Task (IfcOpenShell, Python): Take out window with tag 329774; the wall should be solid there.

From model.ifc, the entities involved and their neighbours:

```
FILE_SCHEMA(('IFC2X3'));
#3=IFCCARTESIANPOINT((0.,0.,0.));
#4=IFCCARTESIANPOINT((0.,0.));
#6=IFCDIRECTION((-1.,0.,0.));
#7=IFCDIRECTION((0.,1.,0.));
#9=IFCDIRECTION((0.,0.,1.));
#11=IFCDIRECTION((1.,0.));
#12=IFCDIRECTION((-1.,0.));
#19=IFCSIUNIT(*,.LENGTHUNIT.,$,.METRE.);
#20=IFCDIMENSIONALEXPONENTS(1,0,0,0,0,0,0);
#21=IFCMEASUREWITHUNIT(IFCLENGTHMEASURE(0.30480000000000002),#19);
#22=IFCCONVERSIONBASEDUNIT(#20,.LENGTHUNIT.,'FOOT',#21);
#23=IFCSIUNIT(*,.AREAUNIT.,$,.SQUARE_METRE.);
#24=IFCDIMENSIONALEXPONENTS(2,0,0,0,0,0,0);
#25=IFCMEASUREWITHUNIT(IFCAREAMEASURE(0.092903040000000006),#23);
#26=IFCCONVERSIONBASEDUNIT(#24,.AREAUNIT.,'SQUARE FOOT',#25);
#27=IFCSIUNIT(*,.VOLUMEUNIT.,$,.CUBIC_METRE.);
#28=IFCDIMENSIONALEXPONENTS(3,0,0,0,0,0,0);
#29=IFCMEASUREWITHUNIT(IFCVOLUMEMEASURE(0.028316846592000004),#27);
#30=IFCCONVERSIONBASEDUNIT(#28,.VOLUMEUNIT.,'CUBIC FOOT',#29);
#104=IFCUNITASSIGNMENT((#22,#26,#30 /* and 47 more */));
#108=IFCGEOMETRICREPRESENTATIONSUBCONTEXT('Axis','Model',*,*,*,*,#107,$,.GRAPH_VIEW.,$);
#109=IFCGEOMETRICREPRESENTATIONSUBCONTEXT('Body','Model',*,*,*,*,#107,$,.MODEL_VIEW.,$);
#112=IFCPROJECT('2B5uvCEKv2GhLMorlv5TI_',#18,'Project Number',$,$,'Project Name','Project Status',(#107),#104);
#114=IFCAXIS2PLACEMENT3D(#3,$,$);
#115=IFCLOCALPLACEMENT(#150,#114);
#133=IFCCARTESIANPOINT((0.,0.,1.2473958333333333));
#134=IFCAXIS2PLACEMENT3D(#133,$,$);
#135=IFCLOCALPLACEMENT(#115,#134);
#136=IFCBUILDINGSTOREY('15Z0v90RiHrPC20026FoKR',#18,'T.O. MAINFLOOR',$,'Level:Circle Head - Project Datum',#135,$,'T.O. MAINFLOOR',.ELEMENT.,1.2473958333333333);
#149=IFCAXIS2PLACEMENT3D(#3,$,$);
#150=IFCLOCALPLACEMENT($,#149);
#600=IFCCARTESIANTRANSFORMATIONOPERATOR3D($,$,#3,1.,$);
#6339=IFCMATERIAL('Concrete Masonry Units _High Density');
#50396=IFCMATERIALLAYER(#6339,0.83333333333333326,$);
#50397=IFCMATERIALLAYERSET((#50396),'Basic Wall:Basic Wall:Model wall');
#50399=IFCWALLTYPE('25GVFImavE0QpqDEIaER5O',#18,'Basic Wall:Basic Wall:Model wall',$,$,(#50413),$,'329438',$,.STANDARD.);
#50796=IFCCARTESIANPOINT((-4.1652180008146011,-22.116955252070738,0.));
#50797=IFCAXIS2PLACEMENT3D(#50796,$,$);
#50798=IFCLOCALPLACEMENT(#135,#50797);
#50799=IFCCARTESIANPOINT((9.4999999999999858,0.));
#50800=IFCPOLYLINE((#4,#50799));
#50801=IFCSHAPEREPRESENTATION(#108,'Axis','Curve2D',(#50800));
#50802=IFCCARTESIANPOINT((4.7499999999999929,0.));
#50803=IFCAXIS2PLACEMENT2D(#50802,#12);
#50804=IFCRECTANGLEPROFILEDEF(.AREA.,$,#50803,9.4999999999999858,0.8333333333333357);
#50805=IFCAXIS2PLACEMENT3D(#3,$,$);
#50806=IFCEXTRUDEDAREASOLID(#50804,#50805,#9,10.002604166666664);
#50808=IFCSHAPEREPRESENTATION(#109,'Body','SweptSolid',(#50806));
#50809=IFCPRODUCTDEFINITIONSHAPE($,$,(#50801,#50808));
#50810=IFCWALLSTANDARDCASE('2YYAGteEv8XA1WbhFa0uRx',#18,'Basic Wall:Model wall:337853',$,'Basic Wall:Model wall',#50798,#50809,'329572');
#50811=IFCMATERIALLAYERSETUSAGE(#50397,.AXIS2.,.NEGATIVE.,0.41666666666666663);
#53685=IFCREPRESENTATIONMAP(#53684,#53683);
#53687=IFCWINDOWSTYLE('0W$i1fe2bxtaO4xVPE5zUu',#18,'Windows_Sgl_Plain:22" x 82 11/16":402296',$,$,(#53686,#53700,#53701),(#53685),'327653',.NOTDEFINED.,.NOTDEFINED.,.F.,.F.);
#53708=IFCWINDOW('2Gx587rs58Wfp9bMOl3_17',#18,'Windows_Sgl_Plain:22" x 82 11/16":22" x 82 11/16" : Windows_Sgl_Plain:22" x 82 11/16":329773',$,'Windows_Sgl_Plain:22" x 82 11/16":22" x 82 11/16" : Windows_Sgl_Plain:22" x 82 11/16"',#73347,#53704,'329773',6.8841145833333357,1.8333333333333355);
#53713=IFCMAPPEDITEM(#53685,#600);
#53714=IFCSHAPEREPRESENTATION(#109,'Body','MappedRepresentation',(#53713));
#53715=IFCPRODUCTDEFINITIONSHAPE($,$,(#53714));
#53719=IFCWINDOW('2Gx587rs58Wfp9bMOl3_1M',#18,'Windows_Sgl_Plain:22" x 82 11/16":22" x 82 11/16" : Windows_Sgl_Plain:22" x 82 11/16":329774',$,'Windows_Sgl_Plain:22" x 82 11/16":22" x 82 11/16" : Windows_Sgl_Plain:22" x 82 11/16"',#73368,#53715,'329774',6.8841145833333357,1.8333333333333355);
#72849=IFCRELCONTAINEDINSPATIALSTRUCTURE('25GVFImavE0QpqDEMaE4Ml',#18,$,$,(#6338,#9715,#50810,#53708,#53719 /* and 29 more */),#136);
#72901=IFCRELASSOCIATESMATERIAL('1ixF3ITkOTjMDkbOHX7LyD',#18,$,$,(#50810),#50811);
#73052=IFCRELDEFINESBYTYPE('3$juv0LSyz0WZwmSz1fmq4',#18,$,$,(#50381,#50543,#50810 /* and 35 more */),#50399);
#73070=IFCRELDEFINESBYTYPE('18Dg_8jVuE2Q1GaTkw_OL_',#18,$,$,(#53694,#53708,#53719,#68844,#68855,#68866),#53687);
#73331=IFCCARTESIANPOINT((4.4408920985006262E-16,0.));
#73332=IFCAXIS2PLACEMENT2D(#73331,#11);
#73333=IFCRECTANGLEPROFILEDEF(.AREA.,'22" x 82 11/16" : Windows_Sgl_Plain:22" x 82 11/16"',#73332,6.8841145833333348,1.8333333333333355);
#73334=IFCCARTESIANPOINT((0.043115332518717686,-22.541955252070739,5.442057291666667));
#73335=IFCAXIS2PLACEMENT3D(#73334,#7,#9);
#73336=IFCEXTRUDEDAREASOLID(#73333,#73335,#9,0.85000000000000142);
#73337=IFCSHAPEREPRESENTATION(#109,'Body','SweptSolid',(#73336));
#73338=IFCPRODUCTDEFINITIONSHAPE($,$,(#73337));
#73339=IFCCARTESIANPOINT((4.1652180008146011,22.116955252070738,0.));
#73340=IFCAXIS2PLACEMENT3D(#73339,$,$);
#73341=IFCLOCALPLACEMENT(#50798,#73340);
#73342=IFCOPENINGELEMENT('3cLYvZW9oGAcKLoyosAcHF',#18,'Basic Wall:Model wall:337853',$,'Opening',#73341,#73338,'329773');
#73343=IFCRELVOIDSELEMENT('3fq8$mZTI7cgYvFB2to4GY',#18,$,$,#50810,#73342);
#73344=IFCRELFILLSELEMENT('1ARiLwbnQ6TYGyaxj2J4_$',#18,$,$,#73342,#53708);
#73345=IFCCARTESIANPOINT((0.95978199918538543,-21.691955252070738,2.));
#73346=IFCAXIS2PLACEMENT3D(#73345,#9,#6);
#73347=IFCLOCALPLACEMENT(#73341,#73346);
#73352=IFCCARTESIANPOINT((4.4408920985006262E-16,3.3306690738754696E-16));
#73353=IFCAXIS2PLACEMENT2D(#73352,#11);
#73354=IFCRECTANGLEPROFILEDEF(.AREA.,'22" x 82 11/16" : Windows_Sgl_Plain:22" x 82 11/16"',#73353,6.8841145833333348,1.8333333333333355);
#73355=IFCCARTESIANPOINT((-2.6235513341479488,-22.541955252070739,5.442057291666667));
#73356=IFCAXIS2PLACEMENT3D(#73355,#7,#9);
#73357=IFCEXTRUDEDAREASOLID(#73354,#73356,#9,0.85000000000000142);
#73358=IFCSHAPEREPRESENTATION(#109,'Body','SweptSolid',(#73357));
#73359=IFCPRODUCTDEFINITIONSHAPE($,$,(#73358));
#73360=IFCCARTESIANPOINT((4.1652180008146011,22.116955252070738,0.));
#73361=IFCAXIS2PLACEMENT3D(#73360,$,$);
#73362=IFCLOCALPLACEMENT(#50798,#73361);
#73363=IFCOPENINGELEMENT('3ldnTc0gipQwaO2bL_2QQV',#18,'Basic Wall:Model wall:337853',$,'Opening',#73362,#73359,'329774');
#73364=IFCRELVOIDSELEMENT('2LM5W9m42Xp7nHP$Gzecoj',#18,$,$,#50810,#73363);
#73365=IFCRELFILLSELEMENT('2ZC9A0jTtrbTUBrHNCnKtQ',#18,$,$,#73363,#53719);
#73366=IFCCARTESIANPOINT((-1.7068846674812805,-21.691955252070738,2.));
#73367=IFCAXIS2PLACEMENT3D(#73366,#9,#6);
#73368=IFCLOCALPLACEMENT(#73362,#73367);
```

```python
import ifcopenshell
import ifcopenshell.api.feature
import ifcopenshell.api.root
import ifcopenshell.geom
import ifcopenshell.util.shape

model = ifcopenshell.open("model.ifc")
settings = ifcopenshell.geom.settings()


def volume(element):
    """Net volume in cubic metres, openings subtracted."""
    shape = ifcopenshell.geom.create_shape(settings, element)
    return ifcopenshell.util.shape.get_volume(shape.geometry)


window = model.by_id(53719)
opening = window.FillsVoids[0].RelatingOpeningElement
wall = opening.VoidsElements[0].RelatingBuildingElement
before = volume(wall)

ifcopenshell.api.root.remove_product(model, product=window)
ifcopenshell.api.feature.remove_feature(model, feature=opening)

after = volume(wall)

print(f"wall volume {before:.3f} -> {after:.3f} m3")

model.write("model_v2.ifc")
```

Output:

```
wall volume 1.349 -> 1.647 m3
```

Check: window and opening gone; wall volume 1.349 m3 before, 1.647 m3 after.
